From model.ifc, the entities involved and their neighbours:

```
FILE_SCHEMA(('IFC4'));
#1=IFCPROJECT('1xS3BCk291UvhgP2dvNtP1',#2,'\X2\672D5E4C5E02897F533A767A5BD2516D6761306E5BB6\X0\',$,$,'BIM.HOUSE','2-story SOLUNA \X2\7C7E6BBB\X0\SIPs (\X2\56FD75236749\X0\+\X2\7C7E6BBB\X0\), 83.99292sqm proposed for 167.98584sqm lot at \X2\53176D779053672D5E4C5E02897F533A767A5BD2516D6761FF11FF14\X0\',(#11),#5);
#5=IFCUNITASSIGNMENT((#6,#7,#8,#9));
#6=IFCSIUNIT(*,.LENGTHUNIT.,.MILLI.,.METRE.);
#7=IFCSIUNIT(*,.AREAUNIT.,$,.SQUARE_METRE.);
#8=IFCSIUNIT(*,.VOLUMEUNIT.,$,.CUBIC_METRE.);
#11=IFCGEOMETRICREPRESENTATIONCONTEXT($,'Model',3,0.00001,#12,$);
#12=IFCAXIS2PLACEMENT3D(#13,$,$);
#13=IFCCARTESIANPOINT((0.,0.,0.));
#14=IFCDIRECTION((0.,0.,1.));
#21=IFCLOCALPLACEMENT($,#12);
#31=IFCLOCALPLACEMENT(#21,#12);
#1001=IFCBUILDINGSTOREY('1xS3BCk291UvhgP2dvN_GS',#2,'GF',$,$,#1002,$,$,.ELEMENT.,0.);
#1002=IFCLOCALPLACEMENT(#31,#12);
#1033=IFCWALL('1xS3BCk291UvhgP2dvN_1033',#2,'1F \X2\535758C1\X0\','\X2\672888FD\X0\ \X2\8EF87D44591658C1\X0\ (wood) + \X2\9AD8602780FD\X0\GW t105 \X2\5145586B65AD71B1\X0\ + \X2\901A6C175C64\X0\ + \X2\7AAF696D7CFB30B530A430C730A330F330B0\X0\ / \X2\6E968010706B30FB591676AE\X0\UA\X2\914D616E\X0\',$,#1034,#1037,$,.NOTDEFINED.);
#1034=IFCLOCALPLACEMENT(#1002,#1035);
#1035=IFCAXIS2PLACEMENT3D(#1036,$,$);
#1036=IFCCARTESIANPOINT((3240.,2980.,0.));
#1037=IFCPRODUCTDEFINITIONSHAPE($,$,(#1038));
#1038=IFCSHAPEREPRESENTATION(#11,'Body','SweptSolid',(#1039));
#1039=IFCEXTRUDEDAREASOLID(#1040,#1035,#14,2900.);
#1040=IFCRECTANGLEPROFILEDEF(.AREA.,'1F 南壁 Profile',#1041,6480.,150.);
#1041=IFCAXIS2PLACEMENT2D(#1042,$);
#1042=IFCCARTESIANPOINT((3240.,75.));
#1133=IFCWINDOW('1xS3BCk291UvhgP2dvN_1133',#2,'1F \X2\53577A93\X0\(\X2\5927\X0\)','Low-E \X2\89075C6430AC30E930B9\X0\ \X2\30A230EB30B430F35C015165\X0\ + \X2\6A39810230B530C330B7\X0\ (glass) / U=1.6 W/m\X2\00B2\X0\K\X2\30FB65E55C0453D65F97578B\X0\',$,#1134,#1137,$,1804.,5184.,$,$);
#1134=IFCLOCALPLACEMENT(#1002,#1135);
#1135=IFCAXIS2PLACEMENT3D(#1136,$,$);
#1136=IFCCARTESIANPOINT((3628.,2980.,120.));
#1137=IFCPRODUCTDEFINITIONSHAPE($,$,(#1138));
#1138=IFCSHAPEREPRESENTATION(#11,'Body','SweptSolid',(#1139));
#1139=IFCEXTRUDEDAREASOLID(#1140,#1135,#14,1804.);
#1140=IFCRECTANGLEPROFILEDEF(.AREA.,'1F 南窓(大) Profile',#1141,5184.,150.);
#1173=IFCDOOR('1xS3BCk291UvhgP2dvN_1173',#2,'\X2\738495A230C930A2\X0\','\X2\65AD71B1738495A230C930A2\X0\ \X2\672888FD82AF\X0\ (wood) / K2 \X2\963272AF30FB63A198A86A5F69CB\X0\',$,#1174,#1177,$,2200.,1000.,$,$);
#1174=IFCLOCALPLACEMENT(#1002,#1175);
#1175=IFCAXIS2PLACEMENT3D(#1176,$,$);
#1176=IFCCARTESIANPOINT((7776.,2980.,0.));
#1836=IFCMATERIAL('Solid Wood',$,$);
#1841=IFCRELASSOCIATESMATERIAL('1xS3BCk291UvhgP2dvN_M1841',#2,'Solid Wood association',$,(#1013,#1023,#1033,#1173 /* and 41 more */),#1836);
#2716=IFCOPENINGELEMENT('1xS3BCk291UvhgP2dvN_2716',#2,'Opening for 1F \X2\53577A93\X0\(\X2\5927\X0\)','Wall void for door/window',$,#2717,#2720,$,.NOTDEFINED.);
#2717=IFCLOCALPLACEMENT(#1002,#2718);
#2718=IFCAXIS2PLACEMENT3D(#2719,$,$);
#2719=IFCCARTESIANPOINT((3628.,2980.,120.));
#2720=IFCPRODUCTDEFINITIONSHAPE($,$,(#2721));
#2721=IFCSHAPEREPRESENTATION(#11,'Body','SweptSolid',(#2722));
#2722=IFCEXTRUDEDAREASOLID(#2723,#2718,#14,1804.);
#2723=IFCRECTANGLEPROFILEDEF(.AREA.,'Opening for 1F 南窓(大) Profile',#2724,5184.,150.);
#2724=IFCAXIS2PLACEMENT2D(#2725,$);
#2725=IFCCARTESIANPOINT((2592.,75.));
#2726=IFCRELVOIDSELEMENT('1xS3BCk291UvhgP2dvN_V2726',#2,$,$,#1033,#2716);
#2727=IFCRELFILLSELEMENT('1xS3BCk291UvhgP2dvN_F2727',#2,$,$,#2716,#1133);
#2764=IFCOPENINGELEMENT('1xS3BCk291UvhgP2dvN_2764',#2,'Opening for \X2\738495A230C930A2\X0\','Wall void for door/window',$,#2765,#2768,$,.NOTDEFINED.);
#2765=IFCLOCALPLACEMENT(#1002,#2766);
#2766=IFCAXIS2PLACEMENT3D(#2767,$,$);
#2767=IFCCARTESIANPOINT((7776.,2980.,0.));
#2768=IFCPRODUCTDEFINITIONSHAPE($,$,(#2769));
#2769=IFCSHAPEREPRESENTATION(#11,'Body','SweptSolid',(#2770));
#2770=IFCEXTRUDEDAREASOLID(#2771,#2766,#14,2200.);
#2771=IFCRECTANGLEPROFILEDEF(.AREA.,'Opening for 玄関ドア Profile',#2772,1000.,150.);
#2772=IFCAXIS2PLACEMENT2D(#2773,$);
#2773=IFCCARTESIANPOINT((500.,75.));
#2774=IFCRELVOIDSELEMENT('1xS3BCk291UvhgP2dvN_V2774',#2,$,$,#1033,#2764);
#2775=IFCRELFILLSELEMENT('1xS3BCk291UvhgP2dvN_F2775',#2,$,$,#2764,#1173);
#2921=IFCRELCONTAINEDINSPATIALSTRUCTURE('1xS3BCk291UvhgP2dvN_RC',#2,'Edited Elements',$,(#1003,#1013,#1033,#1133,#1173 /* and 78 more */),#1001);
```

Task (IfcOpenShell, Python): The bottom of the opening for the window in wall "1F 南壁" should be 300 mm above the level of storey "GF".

```python
import numpy as np
import ifcopenshell
import ifcopenshell.api.geometry
import ifcopenshell.geom
import ifcopenshell.util.element
import ifcopenshell.util.placement
import ifcopenshell.util.shape
import ifcopenshell.util.unit

model = ifcopenshell.open("model.ifc")
unit_scale = ifcopenshell.util.unit.calculate_unit_scale(model)

window = model.by_id(1133)
opening = window.FillsVoids[0].RelatingOpeningElement
storey = ifcopenshell.util.element.get_container(window, ifc_class="IfcBuildingStorey")
level = ifcopenshell.util.placement.get_local_placement(storey.ObjectPlacement)[2, 3]

# The opening's origin need not be at the sill, so measure its lowest point.
shape = ifcopenshell.geom.create_shape(ifcopenshell.geom.settings(), opening)
bottom = ifcopenshell.util.shape.get_shape_bottom_elevation(shape, shape.geometry) / unit_scale
dz = level + 0.3 / unit_scale - bottom

shift = np.array([0.0, 0.0, dz])
# The window is not placed relative to its opening, so move both.
for product in (opening, window):
    matrix = ifcopenshell.util.placement.get_local_placement(product.ObjectPlacement)
    matrix[:3, 3] += shift
    ifcopenshell.api.geometry.edit_object_placement(model, product=product, matrix=matrix, is_si=False)

print(f"moved by {dz * unit_scale:+.3f} m")

model.write("model-out.ifc")
```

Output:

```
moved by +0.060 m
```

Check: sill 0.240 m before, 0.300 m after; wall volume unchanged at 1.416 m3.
